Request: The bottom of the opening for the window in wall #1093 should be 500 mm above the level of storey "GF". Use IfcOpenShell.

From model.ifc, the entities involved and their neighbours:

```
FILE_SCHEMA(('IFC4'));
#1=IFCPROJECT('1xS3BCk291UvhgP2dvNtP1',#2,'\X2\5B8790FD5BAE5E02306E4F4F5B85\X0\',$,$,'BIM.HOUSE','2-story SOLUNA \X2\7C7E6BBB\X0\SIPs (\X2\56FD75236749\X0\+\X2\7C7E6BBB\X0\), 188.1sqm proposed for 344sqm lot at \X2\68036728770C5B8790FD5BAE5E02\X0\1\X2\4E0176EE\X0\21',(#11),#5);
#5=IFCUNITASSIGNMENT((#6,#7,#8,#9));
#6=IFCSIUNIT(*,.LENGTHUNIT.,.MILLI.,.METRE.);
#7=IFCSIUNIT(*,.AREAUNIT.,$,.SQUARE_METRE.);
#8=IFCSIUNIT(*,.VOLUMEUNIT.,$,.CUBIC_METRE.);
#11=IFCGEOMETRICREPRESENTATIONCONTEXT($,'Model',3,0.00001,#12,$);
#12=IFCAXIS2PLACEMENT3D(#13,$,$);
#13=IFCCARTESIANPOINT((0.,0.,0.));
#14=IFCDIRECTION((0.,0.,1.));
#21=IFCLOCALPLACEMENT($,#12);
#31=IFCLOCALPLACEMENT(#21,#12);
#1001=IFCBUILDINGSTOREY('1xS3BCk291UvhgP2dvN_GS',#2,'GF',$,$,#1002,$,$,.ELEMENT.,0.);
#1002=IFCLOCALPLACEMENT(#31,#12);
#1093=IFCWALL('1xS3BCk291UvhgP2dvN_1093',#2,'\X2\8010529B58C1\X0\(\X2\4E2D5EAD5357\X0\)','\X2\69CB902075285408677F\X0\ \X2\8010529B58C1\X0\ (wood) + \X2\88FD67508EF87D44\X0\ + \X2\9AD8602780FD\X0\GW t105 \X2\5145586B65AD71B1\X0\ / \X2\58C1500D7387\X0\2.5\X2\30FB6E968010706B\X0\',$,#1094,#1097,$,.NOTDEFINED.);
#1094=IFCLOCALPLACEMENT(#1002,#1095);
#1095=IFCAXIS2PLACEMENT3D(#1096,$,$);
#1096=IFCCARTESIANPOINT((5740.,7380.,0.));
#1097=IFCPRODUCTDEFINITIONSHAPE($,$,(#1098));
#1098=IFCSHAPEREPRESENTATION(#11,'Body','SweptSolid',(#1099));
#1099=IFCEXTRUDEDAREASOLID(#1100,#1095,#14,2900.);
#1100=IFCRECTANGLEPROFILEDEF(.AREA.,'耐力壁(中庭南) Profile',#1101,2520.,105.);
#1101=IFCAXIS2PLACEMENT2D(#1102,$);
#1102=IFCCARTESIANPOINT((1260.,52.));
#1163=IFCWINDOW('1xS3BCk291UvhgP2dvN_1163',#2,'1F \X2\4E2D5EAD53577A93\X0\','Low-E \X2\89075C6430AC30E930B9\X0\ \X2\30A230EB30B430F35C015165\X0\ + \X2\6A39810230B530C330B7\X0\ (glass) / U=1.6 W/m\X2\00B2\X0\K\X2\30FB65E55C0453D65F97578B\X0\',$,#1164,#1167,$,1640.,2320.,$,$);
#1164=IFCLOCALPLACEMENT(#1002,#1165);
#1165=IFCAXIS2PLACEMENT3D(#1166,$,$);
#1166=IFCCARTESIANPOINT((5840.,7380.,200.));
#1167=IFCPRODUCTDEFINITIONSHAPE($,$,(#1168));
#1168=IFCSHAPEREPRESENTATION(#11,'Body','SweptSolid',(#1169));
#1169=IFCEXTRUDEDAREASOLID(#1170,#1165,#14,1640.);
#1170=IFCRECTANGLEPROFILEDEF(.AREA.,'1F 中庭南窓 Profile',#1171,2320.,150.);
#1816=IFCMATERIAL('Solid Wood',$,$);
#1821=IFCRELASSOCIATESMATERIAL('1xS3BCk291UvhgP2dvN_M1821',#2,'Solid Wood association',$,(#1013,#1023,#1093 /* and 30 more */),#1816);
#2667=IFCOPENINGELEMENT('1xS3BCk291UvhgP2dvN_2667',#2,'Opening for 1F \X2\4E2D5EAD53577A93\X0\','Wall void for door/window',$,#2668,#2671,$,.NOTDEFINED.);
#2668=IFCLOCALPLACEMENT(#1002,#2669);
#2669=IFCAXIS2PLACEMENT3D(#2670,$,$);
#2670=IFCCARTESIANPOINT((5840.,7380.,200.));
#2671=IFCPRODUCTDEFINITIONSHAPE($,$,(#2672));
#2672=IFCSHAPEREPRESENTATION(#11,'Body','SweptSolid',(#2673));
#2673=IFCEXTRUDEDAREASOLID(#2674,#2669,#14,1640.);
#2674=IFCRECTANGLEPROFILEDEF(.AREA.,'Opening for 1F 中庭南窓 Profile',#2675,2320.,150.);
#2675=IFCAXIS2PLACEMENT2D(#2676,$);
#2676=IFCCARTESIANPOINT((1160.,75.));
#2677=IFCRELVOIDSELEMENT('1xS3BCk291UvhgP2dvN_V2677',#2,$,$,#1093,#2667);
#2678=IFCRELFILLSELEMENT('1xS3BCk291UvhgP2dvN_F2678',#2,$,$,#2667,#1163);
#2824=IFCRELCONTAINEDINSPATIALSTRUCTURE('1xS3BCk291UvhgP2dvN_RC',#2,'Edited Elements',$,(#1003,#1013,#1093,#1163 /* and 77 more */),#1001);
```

```python
import numpy as np
import ifcopenshell
import ifcopenshell.api.geometry
import ifcopenshell.geom
import ifcopenshell.util.element
import ifcopenshell.util.placement
import ifcopenshell.util.shape
import ifcopenshell.util.unit

model = ifcopenshell.open("model.ifc")
unit_scale = ifcopenshell.util.unit.calculate_unit_scale(model)

window = model.by_id(1163)
opening = window.FillsVoids[0].RelatingOpeningElement
storey = ifcopenshell.util.element.get_container(window, ifc_class="IfcBuildingStorey")
level = ifcopenshell.util.placement.get_local_placement(storey.ObjectPlacement)[2, 3]

# The opening's origin need not be at the sill, so measure its lowest point.
shape = ifcopenshell.geom.create_shape(ifcopenshell.geom.settings(), opening)
bottom = ifcopenshell.util.shape.get_shape_bottom_elevation(shape, shape.geometry) / unit_scale
dz = level + 0.5 / unit_scale - bottom

shift = np.array([0.0, 0.0, dz])
# The window is not placed relative to its opening, so move both.
for product in (opening, window):
    matrix = ifcopenshell.util.placement.get_local_placement(product.ObjectPlacement)
    matrix[:3, 3] += shift
    ifcopenshell.api.geometry.edit_object_placement(model, product=product, matrix=matrix, is_si=False)

print(f"moved by {dz * unit_scale:+.3f} m")

model.write("model_v2.ifc")
```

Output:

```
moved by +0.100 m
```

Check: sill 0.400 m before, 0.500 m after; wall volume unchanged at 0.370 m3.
